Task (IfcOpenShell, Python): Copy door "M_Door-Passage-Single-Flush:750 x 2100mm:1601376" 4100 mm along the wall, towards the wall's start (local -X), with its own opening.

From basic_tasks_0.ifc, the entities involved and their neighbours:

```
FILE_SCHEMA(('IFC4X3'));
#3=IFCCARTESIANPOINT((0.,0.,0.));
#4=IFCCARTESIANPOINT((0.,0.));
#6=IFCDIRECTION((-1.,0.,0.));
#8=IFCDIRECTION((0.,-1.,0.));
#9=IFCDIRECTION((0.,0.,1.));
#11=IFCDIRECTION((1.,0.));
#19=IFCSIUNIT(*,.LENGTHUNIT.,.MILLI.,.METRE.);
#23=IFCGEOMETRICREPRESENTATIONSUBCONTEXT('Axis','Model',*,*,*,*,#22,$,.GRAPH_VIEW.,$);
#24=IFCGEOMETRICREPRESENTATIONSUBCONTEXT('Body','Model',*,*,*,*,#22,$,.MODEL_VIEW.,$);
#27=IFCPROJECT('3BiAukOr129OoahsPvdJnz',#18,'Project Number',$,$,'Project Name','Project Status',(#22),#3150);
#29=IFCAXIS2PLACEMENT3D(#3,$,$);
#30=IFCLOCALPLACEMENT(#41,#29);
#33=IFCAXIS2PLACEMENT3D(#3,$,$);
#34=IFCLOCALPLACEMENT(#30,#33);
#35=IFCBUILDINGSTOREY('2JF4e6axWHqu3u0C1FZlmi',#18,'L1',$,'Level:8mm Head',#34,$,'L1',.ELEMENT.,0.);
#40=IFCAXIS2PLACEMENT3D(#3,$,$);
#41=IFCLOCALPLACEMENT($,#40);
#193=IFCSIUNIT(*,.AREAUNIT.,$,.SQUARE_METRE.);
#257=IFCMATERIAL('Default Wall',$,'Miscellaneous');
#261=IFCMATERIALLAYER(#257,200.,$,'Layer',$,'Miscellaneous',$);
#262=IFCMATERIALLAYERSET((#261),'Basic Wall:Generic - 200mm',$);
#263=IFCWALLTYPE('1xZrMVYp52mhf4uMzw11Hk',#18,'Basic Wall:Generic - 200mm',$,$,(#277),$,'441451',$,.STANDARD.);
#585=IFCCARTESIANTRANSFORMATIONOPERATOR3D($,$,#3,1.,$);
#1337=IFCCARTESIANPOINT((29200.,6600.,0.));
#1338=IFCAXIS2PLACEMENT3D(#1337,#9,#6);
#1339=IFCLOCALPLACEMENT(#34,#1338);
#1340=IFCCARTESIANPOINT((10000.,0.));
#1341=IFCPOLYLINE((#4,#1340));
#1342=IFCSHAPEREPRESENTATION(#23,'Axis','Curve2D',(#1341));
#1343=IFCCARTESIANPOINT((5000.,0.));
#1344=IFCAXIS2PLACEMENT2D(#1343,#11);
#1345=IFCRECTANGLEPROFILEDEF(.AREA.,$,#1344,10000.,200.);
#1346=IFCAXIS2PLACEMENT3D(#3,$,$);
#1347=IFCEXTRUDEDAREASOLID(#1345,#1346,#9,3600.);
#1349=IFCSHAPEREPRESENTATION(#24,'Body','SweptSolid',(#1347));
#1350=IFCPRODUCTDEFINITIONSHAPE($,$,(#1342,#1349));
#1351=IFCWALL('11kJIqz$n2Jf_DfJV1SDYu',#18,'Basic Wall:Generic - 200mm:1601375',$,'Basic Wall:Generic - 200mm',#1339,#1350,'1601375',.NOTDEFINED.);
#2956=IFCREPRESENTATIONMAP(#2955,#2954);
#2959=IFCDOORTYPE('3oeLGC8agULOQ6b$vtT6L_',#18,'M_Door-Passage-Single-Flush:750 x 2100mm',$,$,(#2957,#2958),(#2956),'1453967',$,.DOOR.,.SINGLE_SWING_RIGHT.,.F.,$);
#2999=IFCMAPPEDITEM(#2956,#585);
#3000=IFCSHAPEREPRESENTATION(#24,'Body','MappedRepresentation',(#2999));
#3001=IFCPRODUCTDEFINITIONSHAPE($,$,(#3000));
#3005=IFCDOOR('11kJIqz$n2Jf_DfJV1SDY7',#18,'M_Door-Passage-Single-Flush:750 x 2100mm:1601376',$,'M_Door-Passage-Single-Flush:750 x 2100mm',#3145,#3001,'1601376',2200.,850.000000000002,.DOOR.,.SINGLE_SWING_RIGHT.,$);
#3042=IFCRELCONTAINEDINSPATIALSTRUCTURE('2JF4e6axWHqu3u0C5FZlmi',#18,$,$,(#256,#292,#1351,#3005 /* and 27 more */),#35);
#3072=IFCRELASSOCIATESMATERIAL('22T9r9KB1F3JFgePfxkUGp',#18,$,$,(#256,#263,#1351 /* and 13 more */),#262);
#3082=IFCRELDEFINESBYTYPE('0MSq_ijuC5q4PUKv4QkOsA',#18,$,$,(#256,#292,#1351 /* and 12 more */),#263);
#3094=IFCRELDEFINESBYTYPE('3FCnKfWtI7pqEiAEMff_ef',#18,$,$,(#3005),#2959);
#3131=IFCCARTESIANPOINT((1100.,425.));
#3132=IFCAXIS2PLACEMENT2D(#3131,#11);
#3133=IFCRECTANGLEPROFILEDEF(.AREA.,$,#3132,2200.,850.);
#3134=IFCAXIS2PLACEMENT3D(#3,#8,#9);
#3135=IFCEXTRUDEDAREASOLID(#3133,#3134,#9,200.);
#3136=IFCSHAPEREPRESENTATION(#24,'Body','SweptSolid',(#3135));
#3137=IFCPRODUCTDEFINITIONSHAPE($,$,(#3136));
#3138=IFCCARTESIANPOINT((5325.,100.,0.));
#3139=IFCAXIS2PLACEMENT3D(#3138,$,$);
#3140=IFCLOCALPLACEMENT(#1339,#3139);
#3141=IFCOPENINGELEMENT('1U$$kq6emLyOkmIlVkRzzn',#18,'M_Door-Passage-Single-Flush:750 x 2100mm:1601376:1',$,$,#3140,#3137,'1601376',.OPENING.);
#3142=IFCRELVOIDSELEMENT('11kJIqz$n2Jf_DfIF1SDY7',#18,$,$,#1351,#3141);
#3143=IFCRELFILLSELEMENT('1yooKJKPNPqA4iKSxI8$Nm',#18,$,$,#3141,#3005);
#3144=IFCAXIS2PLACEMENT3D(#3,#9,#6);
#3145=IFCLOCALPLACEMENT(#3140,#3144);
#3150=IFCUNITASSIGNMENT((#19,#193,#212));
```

```python
import ifcopenshell
import ifcopenshell.api.feature
import ifcopenshell.api.geometry
import ifcopenshell.api.root
import ifcopenshell.geom
import ifcopenshell.util.element
import ifcopenshell.util.placement
import ifcopenshell.util.shape
import ifcopenshell.util.unit

model = ifcopenshell.open("basic_tasks_0.ifc")
unit_scale = ifcopenshell.util.unit.calculate_unit_scale(model)
settings = ifcopenshell.geom.settings()


def volume(element):
    """Net volume in cubic metres, openings subtracted."""
    shape = ifcopenshell.geom.create_shape(settings, element)
    return ifcopenshell.util.shape.get_volume(shape.geometry)


def reuse_history(source, copy):
    """copy_class also copies each property set's owner history, people and application; keep the originals."""
    for rel in copy.IsDefinedBy:
        if rel.is_a("IfcRelDefinesByProperties") and (history := rel.RelatingPropertyDefinition.OwnerHistory):
            rel.RelatingPropertyDefinition.OwnerHistory = source.OwnerHistory
            ifcopenshell.util.element.remove_deep2(model, history)


door = model.by_guid("11kJIqz$n2Jf_DfJV1SDY7")
opening = door.FillsVoids[0].RelatingOpeningElement
wall = opening.VoidsElements[0].RelatingBuildingElement
before = volume(wall)
shift = ifcopenshell.util.placement.get_local_placement(wall.ObjectPlacement)[:3, 0] * -4.1 / unit_scale

# copy_class copies the void relationship, type, container and properties, but no geometry.
new_opening = ifcopenshell.api.root.copy_class(model, product=opening)
new_opening.Representation = ifcopenshell.util.element.copy_deep(
    model, opening.Representation, exclude=["IfcGeometricRepresentationContext", "IfcRepresentationMap"]
)
new_opening.Name = "M_Door-Passage-Single-Flush:750 x 2100mm"
new_opening.Tag = None
new_door = ifcopenshell.api.root.copy_class(model, product=door)
new_door.Representation = ifcopenshell.util.element.copy_deep(
    model, door.Representation, exclude=["IfcGeometricRepresentationContext", "IfcRepresentationMap"]
)
new_door.Name = "M_Door-Passage-Single-Flush:750 x 2100mm"
new_door.Tag = None
reuse_history(door, new_door)
ifcopenshell.api.feature.add_filling(model, opening=new_opening, element=new_door)

for old, new in ((opening, new_opening), (door, new_door)):
    matrix = ifcopenshell.util.placement.get_local_placement(old.ObjectPlacement)
    matrix[:3, 3] += shift
    ifcopenshell.api.geometry.edit_object_placement(model, product=new, matrix=matrix, is_si=False)

after = volume(wall)

print(f"wall volume {before:.3f} -> {after:.3f} m3")

model.write("basic_tasks_0_rev.ifc")
```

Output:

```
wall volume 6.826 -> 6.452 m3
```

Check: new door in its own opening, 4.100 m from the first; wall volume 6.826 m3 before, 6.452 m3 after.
